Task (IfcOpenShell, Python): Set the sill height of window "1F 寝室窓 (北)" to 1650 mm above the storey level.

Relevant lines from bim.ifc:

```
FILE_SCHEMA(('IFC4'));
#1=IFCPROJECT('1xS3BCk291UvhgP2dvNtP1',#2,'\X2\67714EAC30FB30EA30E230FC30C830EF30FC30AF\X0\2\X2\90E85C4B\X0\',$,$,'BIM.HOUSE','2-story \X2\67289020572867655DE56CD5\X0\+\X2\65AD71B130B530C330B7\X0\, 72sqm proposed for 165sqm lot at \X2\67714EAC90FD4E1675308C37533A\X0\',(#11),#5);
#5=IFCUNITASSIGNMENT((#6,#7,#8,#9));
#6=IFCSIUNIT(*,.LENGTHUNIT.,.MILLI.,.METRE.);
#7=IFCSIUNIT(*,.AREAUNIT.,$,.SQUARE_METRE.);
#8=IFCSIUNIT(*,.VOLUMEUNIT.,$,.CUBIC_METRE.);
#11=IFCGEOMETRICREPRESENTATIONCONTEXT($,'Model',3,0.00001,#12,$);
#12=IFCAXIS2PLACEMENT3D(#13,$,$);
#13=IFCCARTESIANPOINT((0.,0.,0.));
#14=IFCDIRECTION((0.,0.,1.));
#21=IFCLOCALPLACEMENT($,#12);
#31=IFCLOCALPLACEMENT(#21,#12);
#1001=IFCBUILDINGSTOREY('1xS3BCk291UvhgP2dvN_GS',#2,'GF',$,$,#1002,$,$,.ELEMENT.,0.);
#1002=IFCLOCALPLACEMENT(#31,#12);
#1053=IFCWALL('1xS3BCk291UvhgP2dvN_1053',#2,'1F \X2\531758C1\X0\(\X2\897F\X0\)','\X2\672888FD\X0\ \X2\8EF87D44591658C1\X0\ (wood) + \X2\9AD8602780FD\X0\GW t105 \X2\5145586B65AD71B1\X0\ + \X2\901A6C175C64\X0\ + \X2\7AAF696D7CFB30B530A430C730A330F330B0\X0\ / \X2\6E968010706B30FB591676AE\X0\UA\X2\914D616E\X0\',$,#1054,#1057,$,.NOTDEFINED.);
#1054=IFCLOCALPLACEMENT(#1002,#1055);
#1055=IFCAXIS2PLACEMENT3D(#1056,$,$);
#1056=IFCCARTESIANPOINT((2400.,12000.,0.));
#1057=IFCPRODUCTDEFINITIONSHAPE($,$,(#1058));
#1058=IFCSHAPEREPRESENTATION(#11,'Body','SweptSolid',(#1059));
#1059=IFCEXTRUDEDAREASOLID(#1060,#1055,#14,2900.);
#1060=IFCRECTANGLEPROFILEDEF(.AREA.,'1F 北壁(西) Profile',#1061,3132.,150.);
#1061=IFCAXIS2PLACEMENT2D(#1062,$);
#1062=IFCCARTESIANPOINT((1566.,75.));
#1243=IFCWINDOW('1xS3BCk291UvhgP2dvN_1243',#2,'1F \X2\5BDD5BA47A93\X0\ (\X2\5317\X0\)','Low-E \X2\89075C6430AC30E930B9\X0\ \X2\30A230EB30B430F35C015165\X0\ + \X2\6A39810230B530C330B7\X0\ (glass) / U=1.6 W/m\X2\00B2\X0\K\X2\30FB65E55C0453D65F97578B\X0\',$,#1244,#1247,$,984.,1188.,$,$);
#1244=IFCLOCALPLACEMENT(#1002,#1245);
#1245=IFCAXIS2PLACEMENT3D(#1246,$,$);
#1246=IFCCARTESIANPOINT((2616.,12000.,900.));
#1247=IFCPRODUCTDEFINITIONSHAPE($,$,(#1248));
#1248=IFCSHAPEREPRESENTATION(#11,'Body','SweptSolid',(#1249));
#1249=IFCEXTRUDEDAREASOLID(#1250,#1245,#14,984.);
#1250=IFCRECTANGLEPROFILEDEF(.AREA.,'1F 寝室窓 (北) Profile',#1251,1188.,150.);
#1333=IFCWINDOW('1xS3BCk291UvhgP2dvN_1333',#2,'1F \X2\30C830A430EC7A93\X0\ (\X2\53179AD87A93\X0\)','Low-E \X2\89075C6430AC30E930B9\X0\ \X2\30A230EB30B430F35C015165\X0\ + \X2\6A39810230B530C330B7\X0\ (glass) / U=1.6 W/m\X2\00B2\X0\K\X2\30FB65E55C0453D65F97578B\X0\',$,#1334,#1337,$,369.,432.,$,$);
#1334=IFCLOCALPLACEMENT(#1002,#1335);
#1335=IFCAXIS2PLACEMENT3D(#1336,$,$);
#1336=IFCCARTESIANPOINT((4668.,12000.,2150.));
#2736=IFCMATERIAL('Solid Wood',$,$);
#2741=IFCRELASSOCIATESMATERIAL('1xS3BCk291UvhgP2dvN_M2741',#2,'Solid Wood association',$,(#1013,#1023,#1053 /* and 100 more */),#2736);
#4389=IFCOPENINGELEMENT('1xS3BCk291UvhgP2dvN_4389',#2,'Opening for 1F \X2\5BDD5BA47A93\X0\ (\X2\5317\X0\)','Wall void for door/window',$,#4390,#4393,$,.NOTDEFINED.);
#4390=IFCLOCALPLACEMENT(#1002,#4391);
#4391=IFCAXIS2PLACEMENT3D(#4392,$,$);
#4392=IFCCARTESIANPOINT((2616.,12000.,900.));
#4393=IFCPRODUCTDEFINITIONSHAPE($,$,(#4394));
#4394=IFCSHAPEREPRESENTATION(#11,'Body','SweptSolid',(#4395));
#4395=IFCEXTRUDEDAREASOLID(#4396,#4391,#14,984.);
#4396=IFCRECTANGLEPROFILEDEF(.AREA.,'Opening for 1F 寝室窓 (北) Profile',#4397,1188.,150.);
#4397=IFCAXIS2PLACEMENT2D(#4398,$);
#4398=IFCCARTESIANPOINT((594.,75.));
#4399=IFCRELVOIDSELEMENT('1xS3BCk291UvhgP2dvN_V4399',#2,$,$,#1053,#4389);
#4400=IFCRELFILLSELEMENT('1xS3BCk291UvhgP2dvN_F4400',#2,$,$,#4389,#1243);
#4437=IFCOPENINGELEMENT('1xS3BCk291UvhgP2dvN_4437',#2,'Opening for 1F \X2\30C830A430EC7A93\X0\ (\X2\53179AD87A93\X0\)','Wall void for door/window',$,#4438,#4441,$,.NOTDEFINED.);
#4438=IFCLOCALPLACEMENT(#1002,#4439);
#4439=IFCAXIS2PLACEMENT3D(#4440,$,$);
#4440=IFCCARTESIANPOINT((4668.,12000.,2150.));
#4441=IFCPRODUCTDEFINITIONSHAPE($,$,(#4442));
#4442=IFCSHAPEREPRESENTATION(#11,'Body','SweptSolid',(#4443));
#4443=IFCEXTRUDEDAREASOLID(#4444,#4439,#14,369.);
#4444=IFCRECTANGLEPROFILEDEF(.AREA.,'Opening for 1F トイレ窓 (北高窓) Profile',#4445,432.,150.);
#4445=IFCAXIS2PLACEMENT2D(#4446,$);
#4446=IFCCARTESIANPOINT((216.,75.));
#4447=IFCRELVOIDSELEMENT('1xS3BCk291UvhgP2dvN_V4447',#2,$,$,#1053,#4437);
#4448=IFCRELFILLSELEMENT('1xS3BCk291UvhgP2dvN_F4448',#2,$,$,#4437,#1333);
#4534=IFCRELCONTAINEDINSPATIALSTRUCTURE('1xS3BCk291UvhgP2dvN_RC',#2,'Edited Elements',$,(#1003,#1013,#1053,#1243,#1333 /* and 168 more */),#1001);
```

```python
import numpy as np
import ifcopenshell
import ifcopenshell.api.geometry
import ifcopenshell.geom
import ifcopenshell.util.element
import ifcopenshell.util.placement
import ifcopenshell.util.shape
import ifcopenshell.util.unit

model = ifcopenshell.open("bim.ifc")
unit_scale = ifcopenshell.util.unit.calculate_unit_scale(model)

window = model.by_guid("1xS3BCk291UvhgP2dvN_1243")
opening = window.FillsVoids[0].RelatingOpeningElement
storey = ifcopenshell.util.element.get_container(window, ifc_class="IfcBuildingStorey")
level = ifcopenshell.util.placement.get_local_placement(storey.ObjectPlacement)[2, 3]

# The opening's origin need not be at the sill, so measure its lowest point.
shape = ifcopenshell.geom.create_shape(ifcopenshell.geom.settings(), opening)
bottom = ifcopenshell.util.shape.get_shape_bottom_elevation(shape, shape.geometry) / unit_scale
dz = level + 1650.0 - bottom

shift = np.array([0.0, 0.0, dz])
# The window is not placed relative to its opening, so move both.
for product in (opening, window):
    matrix = ifcopenshell.util.placement.get_local_placement(product.ObjectPlacement)
    matrix[:3, 3] += shift
    ifcopenshell.api.geometry.edit_object_placement(model, product=product, matrix=matrix, is_si=False)

print(f"moved by {dz * unit_scale:+.3f} m")

model.write("bim_updated.ifc")
```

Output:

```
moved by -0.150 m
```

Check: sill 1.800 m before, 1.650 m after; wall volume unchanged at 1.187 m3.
